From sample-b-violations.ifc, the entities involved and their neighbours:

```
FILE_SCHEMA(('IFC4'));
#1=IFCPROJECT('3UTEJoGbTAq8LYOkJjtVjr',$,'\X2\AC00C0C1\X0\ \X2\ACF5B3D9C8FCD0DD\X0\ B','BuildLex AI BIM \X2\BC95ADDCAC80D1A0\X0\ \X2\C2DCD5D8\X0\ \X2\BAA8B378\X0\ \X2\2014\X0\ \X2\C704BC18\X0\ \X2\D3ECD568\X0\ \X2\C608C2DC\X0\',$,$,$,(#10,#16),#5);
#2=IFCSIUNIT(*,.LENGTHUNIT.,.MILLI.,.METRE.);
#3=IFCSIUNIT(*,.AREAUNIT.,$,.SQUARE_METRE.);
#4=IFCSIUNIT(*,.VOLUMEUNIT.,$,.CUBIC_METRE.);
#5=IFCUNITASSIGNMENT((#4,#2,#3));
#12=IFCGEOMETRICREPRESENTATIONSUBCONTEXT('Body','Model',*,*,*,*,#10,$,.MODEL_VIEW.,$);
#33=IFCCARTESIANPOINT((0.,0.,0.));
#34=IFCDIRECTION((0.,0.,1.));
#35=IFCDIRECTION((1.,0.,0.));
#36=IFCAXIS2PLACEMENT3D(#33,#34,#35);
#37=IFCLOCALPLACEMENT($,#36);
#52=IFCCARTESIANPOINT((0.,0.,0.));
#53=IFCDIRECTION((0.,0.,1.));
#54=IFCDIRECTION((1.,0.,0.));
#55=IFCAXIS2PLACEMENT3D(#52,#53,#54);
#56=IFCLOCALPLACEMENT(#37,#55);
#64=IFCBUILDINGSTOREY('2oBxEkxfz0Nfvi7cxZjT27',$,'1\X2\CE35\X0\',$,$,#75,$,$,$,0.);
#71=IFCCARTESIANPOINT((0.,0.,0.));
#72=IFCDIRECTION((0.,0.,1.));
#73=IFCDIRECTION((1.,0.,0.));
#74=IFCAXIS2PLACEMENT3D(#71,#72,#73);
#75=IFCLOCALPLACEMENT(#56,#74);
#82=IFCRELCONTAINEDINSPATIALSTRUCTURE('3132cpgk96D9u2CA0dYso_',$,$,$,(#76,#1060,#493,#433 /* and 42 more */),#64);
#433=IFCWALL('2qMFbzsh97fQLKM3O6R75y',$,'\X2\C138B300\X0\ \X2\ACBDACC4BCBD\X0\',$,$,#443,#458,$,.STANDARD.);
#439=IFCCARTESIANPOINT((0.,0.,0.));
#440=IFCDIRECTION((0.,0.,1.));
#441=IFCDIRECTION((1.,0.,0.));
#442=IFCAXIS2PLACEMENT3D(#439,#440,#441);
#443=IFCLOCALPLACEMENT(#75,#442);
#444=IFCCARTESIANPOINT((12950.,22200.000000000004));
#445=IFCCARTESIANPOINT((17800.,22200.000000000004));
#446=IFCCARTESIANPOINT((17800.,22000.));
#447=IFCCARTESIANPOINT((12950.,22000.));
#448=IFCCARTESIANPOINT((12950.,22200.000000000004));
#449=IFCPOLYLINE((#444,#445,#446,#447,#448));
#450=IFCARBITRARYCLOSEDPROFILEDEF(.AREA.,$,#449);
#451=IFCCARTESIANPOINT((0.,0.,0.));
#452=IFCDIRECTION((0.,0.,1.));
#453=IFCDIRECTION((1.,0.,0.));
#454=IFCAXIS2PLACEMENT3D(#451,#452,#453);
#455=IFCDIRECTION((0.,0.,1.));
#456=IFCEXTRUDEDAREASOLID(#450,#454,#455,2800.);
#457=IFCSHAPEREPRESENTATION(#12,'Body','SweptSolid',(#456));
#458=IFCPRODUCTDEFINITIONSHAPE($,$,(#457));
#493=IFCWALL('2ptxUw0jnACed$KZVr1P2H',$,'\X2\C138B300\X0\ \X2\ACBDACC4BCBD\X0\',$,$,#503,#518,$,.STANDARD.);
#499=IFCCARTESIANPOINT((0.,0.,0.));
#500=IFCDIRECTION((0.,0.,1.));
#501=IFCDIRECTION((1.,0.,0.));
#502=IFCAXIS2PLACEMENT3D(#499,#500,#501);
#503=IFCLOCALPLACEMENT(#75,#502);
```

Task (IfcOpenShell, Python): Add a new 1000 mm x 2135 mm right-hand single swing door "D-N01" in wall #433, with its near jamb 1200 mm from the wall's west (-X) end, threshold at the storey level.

```python
import numpy as np
import ifcopenshell
import ifcopenshell.api.feature
import ifcopenshell.api.geometry
import ifcopenshell.api.root
import ifcopenshell.api.spatial
import ifcopenshell.geom
import ifcopenshell.util.element
import ifcopenshell.util.placement
import ifcopenshell.util.representation
import ifcopenshell.util.shape
import ifcopenshell.util.unit

model = ifcopenshell.open("sample-b-violations.ifc")
unit_scale = ifcopenshell.util.unit.calculate_unit_scale(model)
settings = ifcopenshell.geom.settings()


def volume(element):
    """Net volume in cubic metres, openings subtracted."""
    shape = ifcopenshell.geom.create_shape(settings, element)
    return ifcopenshell.util.shape.get_volume(shape.geometry)


wall = model.by_guid("2qMFbzsh97fQLKM3O6R75y")
storey = ifcopenshell.util.element.get_container(wall, ifc_class="IfcBuildingStorey")
context = ifcopenshell.util.representation.get_context(model, "Model", "Body", "MODEL_VIEW")
before = volume(wall)

width, height, from_end, sill = 1, 2.135, 1.2, 0.0  # metres

# The wall runs along its own X axis, and the end named is its -X end.
wall_shape = ifcopenshell.geom.create_shape(settings, wall)
x, y, z = ifcopenshell.util.shape.get_vertices(wall_shape.geometry).T
start = x.min() + from_end
face, thickness = float(y.min()), float(y.max() - y.min())
wall_matrix = ifcopenshell.util.placement.get_local_placement(wall.ObjectPlacement)
level = ifcopenshell.util.placement.get_local_placement(storey.ObjectPlacement)[2, 3]


def in_wall(x, y):
    """Placement at x, y metres in the wall's axes, at sill height."""
    matrix = wall_matrix.copy()
    matrix[:, 3] = wall_matrix @ np.array([x / unit_scale, y / unit_scale, 0.0, 1.0])
    matrix[2, 3] = level + sill / unit_scale
    return matrix


# Opening: a box that overshoots both wall faces by 50 mm.
opening = ifcopenshell.api.root.create_entity(model, ifc_class="IfcOpeningElement", predefined_type="OPENING")
box = ifcopenshell.api.geometry.add_wall_representation(
    model, context=context, length=width, height=height, thickness=thickness + 0.1
)
ifcopenshell.api.geometry.assign_representation(model, product=opening, representation=box)
ifcopenshell.api.geometry.edit_object_placement(model, product=opening, matrix=in_wall(start, face - 0.05), is_si=False)
ifcopenshell.api.feature.add_feature(model, feature=opening, element=wall)

door = ifcopenshell.api.root.create_entity(model, ifc_class="IfcDoor", name="D-N01", predefined_type="DOOR")
door.OverallWidth, door.OverallHeight = width / unit_scale, height / unit_scale
door.OperationType = "SINGLE_SWING_RIGHT"
body = ifcopenshell.api.geometry.add_door_representation(
    model,
    context=context,
    overall_width=door.OverallWidth,
    overall_height=door.OverallHeight,
    operation_type="SINGLE_SWING_RIGHT",
    lining_properties={"LiningDepth": thickness / unit_scale, "ThresholdDepth": thickness / unit_scale},
)
ifcopenshell.api.geometry.assign_representation(model, product=door, representation=body)
ifcopenshell.api.spatial.assign_container(model, products=[door], relating_structure=storey)
ifcopenshell.api.feature.add_filling(model, opening=opening, element=door)

# The lining spans the wall, so the door starts at the wall face.
ifcopenshell.api.geometry.edit_object_placement(model, product=door, matrix=in_wall(start, face), is_si=False)

after = volume(wall)

print(f"wall volume {before:.3f} -> {after:.3f} m3")

model.write("sample-b-violations_updated.ifc")
```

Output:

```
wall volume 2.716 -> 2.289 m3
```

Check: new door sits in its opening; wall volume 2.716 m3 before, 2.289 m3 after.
